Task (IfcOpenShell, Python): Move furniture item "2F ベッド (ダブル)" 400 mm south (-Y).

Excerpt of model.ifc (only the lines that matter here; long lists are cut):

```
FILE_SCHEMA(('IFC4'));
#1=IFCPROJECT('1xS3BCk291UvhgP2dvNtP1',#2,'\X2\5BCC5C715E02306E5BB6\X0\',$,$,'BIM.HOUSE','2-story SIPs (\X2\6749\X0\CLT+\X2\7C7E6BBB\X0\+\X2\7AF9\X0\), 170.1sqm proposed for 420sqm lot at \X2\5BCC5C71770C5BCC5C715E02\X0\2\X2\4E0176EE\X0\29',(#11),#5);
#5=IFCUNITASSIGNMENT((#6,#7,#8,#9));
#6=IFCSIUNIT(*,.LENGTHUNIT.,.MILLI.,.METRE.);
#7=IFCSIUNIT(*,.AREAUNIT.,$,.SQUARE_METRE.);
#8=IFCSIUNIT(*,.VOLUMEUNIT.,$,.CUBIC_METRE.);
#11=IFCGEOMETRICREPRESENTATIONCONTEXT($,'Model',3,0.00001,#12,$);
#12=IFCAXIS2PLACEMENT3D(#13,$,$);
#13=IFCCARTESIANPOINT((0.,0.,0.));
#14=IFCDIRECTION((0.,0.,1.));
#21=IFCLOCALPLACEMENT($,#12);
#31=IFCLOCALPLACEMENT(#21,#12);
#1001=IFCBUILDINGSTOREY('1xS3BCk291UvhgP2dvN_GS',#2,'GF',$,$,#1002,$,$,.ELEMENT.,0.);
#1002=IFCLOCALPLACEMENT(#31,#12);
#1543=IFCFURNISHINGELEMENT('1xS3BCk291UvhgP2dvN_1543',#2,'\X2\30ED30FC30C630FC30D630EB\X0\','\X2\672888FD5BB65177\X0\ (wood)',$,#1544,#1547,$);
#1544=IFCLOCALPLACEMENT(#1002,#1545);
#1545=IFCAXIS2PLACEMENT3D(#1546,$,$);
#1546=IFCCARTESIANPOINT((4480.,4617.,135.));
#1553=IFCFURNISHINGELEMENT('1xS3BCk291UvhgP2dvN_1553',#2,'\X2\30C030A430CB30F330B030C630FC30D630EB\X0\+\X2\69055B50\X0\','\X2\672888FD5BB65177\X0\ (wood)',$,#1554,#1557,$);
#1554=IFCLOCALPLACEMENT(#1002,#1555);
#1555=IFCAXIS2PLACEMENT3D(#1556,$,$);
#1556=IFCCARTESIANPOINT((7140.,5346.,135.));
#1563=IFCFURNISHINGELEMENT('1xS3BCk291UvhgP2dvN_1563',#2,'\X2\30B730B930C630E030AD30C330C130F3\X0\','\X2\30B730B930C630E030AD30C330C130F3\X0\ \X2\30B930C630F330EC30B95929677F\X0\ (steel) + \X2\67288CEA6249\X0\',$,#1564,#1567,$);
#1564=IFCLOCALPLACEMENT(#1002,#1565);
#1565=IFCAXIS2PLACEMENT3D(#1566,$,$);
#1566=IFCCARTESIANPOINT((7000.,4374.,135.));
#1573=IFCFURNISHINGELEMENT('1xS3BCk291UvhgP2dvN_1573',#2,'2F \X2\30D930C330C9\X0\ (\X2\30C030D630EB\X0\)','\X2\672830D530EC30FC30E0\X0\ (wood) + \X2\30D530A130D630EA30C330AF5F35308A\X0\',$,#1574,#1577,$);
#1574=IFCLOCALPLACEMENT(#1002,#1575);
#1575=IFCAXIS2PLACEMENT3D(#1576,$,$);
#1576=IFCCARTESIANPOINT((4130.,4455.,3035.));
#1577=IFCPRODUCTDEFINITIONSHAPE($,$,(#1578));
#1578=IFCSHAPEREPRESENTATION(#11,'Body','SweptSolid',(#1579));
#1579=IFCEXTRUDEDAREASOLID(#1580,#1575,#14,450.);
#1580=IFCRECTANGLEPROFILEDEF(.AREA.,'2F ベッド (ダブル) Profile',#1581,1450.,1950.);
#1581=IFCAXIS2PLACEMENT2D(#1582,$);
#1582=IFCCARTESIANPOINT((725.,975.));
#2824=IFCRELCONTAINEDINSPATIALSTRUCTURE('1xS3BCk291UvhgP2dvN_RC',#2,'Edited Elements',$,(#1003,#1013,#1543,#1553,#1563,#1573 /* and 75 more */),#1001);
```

```python
import ifcopenshell
import ifcopenshell.api.geometry
import ifcopenshell.util.placement
import ifcopenshell.util.unit

model = ifcopenshell.open("model.ifc")
unit_scale = ifcopenshell.util.unit.calculate_unit_scale(model)

item = model.by_guid("1xS3BCk291UvhgP2dvN_1573")
matrix = ifcopenshell.util.placement.get_local_placement(item.ObjectPlacement)
matrix[1, 3] -= 0.4 / unit_scale
ifcopenshell.api.geometry.edit_object_placement(model, product=item, matrix=matrix, is_si=False)

print(ifcopenshell.util.placement.get_local_placement(item.ObjectPlacement).round(3) + 0.0)

model.write("model_v2.ifc")
```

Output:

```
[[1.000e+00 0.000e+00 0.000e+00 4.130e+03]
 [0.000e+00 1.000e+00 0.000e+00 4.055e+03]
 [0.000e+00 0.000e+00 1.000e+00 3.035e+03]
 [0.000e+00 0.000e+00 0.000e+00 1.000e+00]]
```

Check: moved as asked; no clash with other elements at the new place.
